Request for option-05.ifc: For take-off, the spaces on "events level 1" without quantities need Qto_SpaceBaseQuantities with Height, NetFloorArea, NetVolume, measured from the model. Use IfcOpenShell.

First a look at what the model holds.

```python
import ifcopenshell
import ifcopenshell.util.element
import ifcopenshell.util.unit

model = ifcopenshell.open("option-05.ifc")
print(model.schema)
for unit_type in ("LENGTHUNIT", "AREAUNIT", "VOLUMEUNIT"):
    print(unit_type, ifcopenshell.util.unit.calculate_unit_scale(model, unit_type))
storey = next(s for s in model.by_type("IfcBuildingStorey") if s.Name == "events level 1")
spaces = [e for e in ifcopenshell.util.element.get_decomposition(storey) if e.is_a("IfcSpace")]
for e in sorted(spaces, key=lambda e: e.id()):
    print(e.id(), e.is_a(), e.Name, list(ifcopenshell.util.element.get_psets(e, qtos_only=True)), sep=" | ")
```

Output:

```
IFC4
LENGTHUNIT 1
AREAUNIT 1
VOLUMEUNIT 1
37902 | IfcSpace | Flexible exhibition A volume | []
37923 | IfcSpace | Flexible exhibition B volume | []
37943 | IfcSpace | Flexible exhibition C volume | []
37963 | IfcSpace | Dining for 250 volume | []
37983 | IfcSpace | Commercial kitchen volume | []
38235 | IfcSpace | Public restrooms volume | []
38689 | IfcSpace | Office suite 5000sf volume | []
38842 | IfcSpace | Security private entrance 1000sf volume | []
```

```python
import ifcopenshell
import ifcopenshell.api.pset
import ifcopenshell.geom
import ifcopenshell.util.element
import ifcopenshell.util.shape
import ifcopenshell.util.unit

model = ifcopenshell.open("option-05.ifc")
unit_scale = ifcopenshell.util.unit.calculate_unit_scale(model)
area_scale = ifcopenshell.util.unit.calculate_unit_scale(model, "AREAUNIT")
volume_scale = ifcopenshell.util.unit.calculate_unit_scale(model, "VOLUMEUNIT")
settings = ifcopenshell.geom.settings()

storey = next(s for s in model.by_type("IfcBuildingStorey") if s.Name == "events level 1")
spaces = [e for e in ifcopenshell.util.element.get_decomposition(storey) if e.is_a("IfcSpace")]

for e in sorted(spaces, key=lambda e: e.id()):
    if ifcopenshell.util.element.get_psets(e, qtos_only=True, should_inherit=False):
        continue
    # Geometry comes back in metres, in the element's own axes.
    shape = ifcopenshell.geom.create_shape(settings, e)
    values = {
        "Height": ifcopenshell.util.shape.get_z(shape.geometry) / unit_scale,
        "NetFloorArea": ifcopenshell.util.shape.get_footprint_area(shape.geometry) / area_scale,
        "NetVolume": ifcopenshell.util.shape.get_volume(shape.geometry) / volume_scale,
    }
    qto = ifcopenshell.api.pset.add_qto(model, product=e, name="Qto_SpaceBaseQuantities")
    ifcopenshell.api.pset.edit_qto(model, qto=qto, properties=values)
    print(e.id(), {k: round(v, 3) for k, v in values.items()})

model.write("option-05_updated.ifc")
```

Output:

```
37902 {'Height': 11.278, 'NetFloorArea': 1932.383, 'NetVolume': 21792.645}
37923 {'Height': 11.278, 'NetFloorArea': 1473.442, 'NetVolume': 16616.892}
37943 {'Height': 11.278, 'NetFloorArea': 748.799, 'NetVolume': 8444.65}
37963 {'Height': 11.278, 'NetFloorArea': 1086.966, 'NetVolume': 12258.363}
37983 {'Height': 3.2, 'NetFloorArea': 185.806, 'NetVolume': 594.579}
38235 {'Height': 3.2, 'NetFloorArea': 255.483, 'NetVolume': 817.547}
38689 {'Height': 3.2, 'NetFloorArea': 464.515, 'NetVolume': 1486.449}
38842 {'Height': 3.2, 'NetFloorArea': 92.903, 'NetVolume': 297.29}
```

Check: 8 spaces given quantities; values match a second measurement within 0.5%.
